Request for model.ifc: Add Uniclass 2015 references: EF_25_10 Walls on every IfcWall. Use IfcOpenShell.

First a look at what the model holds.

```python
import ifcopenshell

model = ifcopenshell.open("model.ifc")
print(model.schema)
print("classifications:", [c.Name for c in model.by_type("IfcClassification")])
for ifc_class in ("IfcDoor", "IfcRoof", "IfcStair", "IfcWall", "IfcWindow"):
    print(ifc_class, len(model.by_type(ifc_class)))
```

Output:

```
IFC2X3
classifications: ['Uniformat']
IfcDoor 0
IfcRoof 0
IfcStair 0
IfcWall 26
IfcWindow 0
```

```python
import ifcopenshell
import ifcopenshell.api.classification

model = ifcopenshell.open("model.ifc")

# IFC2X3 requires Source and Edition and has no link from the project to the system.
system = model.create_entity("IfcClassification", Source="NBS", Edition="2015", Name="Uniclass 2015")

codes = {
    "IfcWall": ("EF_25_10", "Walls"),
}
for ifc_class, (code, name) in codes.items():
    products = model.by_type(ifc_class)
    ifcopenshell.api.classification.add_reference(
        model, products=products, classification=system, identification=code, name=name
    )
    print(code, len(products))

model.write("model_updated.ifc")
```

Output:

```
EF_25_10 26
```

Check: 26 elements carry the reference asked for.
